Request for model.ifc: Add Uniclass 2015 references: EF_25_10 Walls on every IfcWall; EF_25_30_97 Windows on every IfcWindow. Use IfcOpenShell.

First a look at what the model holds.

```python
import ifcopenshell

model = ifcopenshell.open("model.ifc")
print(model.schema)
print("classifications:", [c.Name for c in model.by_type("IfcClassification")])
for ifc_class in ("IfcDoor", "IfcRoof", "IfcStair", "IfcWall", "IfcWindow"):
    print(ifc_class, len(model.by_type(ifc_class)))
```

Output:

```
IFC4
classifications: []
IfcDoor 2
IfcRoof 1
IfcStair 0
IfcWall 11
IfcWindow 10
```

```python
import ifcopenshell
import ifcopenshell.api.classification

model = ifcopenshell.open("model.ifc")

system = ifcopenshell.api.classification.add_classification(model, classification="Uniclass 2015")

codes = {
    "IfcWall": ("EF_25_10", "Walls"),
    "IfcWindow": ("EF_25_30_97", "Windows"),
}
for ifc_class, (code, name) in codes.items():
    products = model.by_type(ifc_class)
    ifcopenshell.api.classification.add_reference(
        model, products=products, classification=system, identification=code, name=name
    )
    print(code, len(products))

model.write("model_rev.ifc")
```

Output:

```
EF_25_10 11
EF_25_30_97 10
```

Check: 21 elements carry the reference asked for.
